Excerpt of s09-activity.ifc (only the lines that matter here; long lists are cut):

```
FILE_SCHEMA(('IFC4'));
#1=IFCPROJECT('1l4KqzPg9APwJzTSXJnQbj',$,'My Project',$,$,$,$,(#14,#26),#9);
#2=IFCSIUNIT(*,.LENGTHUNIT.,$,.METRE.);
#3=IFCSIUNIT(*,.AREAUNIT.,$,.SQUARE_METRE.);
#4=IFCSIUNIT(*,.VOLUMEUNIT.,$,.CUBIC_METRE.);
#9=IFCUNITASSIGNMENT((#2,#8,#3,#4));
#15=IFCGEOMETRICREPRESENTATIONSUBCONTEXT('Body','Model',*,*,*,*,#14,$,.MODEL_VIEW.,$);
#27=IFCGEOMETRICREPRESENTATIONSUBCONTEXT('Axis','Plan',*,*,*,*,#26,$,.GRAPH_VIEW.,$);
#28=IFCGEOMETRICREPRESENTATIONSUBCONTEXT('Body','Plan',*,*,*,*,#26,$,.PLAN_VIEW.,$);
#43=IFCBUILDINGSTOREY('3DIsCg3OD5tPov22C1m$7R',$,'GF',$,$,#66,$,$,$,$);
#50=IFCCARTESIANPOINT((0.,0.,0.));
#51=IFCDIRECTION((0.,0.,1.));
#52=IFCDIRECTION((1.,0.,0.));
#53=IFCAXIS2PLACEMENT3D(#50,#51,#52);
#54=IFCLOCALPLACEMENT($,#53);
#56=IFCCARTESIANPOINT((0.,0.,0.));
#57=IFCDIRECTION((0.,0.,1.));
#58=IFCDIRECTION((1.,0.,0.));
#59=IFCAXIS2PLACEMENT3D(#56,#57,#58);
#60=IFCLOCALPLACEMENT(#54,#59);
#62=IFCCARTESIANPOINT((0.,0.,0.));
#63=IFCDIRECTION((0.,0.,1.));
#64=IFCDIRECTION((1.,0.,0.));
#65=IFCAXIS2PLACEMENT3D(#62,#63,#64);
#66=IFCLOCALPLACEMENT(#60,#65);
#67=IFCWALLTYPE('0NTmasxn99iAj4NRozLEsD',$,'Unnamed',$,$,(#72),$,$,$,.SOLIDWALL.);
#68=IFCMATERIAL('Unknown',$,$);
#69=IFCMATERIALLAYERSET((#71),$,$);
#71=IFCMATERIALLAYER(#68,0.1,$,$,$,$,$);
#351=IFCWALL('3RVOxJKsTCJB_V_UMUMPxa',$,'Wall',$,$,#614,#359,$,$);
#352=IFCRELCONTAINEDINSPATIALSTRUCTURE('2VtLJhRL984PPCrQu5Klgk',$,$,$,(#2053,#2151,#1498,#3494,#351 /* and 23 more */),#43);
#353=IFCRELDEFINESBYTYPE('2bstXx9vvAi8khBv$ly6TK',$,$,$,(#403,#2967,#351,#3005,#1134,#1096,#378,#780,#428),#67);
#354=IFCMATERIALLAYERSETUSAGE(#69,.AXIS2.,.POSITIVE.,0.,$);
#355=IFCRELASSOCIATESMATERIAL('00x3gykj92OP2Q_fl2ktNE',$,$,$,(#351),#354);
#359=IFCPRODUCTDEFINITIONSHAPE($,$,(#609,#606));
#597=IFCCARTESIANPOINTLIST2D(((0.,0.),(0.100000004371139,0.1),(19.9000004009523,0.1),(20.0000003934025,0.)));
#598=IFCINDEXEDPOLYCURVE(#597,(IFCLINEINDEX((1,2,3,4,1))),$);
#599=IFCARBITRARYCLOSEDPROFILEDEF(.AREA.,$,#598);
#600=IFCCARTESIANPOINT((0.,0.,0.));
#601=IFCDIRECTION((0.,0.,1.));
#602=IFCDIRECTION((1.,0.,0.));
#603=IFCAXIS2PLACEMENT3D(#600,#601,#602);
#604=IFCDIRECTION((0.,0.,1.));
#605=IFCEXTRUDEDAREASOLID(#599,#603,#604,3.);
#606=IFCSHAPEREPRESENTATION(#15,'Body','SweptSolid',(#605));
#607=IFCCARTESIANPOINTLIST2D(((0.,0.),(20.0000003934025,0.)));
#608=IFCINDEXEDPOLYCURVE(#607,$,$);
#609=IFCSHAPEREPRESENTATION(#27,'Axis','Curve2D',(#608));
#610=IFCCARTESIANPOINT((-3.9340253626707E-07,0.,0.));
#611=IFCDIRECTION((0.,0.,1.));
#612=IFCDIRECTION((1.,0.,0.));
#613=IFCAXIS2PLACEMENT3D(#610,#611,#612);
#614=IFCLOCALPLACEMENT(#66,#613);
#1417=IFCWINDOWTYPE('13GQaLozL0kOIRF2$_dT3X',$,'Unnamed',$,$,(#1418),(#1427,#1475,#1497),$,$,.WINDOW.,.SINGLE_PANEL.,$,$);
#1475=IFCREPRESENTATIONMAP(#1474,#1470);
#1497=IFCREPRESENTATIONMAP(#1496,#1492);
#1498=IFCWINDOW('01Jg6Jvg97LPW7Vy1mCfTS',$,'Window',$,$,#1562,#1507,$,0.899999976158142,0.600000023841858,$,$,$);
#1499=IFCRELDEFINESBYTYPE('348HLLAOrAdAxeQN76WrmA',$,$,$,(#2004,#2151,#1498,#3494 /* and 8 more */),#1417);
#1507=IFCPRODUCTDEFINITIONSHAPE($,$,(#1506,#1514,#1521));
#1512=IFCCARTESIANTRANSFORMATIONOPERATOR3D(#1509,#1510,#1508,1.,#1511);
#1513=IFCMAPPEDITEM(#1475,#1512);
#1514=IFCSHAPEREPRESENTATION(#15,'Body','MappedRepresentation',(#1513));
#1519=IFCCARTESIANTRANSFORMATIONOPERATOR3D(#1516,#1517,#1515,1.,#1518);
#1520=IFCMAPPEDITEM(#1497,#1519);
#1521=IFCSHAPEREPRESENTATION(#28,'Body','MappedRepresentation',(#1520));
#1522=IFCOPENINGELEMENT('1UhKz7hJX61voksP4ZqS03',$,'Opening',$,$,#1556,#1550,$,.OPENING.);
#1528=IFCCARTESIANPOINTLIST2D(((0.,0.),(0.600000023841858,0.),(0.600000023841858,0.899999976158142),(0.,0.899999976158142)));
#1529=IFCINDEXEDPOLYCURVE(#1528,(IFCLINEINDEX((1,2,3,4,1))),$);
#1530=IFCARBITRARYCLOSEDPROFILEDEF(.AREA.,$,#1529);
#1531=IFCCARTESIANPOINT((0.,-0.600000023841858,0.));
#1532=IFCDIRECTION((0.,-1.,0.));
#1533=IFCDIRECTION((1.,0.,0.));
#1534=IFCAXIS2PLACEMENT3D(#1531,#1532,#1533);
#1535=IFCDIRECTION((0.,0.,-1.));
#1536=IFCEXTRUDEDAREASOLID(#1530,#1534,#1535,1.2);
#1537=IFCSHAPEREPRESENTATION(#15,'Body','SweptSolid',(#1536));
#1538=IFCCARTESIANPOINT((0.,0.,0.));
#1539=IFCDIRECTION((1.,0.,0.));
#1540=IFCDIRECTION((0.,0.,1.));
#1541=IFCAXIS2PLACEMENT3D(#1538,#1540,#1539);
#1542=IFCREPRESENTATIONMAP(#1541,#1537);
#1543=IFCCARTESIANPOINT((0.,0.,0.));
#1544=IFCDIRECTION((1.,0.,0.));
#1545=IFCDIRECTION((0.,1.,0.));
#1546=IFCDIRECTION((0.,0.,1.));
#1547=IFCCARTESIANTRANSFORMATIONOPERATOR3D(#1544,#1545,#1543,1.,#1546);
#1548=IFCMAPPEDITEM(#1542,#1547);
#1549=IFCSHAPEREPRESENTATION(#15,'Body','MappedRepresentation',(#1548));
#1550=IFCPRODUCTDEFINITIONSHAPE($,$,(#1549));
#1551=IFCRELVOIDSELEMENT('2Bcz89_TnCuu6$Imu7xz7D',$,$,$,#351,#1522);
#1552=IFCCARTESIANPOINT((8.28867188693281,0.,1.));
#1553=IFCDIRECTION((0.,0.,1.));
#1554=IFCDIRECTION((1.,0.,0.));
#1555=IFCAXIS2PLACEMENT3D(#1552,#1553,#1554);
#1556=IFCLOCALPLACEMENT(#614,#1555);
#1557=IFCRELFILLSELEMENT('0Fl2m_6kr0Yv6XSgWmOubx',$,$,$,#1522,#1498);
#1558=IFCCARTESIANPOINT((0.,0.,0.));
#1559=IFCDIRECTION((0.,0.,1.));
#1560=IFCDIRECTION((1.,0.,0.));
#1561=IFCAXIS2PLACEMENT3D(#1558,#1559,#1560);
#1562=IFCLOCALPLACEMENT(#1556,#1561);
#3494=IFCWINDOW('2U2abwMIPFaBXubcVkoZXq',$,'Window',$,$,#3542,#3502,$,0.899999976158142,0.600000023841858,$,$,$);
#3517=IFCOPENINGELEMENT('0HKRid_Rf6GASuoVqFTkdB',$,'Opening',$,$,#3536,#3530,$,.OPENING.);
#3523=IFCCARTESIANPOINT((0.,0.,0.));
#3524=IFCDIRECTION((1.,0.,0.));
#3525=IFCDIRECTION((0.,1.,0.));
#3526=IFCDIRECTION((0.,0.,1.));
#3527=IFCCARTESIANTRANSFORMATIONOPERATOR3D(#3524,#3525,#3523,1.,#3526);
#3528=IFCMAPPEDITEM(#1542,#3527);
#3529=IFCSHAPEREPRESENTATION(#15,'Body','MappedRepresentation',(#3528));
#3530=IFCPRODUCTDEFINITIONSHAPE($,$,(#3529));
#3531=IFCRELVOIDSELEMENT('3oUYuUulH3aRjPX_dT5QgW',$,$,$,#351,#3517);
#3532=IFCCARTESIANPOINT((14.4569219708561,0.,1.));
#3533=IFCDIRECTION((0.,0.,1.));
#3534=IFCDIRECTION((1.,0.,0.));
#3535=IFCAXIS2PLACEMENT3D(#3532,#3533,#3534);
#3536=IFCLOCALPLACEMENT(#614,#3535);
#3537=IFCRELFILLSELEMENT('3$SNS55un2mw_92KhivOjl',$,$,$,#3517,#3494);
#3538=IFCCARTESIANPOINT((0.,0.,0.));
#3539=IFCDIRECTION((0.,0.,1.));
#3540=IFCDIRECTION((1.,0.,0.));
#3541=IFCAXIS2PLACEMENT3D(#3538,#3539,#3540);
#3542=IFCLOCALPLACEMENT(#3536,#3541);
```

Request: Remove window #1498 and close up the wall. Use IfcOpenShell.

```python
import ifcopenshell
import ifcopenshell.api.feature
import ifcopenshell.api.root
import ifcopenshell.geom
import ifcopenshell.util.shape

model = ifcopenshell.open("s09-activity.ifc")
settings = ifcopenshell.geom.settings()


def volume(element):
    """Net volume in cubic metres, openings subtracted."""
    shape = ifcopenshell.geom.create_shape(settings, element)
    return ifcopenshell.util.shape.get_volume(shape.geometry)


window = model.by_guid("01Jg6Jvg97LPW7Vy1mCfTS")
opening = window.FillsVoids[0].RelatingOpeningElement
wall = opening.VoidsElements[0].RelatingBuildingElement
before = volume(wall)

ifcopenshell.api.root.remove_product(model, product=window)
ifcopenshell.api.feature.remove_feature(model, feature=opening)

after = volume(wall)

print(f"wall volume {before:.3f} -> {after:.3f} m3")

model.write("s09-activity_updated.ifc")
```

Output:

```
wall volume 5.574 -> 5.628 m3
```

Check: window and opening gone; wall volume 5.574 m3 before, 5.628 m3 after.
